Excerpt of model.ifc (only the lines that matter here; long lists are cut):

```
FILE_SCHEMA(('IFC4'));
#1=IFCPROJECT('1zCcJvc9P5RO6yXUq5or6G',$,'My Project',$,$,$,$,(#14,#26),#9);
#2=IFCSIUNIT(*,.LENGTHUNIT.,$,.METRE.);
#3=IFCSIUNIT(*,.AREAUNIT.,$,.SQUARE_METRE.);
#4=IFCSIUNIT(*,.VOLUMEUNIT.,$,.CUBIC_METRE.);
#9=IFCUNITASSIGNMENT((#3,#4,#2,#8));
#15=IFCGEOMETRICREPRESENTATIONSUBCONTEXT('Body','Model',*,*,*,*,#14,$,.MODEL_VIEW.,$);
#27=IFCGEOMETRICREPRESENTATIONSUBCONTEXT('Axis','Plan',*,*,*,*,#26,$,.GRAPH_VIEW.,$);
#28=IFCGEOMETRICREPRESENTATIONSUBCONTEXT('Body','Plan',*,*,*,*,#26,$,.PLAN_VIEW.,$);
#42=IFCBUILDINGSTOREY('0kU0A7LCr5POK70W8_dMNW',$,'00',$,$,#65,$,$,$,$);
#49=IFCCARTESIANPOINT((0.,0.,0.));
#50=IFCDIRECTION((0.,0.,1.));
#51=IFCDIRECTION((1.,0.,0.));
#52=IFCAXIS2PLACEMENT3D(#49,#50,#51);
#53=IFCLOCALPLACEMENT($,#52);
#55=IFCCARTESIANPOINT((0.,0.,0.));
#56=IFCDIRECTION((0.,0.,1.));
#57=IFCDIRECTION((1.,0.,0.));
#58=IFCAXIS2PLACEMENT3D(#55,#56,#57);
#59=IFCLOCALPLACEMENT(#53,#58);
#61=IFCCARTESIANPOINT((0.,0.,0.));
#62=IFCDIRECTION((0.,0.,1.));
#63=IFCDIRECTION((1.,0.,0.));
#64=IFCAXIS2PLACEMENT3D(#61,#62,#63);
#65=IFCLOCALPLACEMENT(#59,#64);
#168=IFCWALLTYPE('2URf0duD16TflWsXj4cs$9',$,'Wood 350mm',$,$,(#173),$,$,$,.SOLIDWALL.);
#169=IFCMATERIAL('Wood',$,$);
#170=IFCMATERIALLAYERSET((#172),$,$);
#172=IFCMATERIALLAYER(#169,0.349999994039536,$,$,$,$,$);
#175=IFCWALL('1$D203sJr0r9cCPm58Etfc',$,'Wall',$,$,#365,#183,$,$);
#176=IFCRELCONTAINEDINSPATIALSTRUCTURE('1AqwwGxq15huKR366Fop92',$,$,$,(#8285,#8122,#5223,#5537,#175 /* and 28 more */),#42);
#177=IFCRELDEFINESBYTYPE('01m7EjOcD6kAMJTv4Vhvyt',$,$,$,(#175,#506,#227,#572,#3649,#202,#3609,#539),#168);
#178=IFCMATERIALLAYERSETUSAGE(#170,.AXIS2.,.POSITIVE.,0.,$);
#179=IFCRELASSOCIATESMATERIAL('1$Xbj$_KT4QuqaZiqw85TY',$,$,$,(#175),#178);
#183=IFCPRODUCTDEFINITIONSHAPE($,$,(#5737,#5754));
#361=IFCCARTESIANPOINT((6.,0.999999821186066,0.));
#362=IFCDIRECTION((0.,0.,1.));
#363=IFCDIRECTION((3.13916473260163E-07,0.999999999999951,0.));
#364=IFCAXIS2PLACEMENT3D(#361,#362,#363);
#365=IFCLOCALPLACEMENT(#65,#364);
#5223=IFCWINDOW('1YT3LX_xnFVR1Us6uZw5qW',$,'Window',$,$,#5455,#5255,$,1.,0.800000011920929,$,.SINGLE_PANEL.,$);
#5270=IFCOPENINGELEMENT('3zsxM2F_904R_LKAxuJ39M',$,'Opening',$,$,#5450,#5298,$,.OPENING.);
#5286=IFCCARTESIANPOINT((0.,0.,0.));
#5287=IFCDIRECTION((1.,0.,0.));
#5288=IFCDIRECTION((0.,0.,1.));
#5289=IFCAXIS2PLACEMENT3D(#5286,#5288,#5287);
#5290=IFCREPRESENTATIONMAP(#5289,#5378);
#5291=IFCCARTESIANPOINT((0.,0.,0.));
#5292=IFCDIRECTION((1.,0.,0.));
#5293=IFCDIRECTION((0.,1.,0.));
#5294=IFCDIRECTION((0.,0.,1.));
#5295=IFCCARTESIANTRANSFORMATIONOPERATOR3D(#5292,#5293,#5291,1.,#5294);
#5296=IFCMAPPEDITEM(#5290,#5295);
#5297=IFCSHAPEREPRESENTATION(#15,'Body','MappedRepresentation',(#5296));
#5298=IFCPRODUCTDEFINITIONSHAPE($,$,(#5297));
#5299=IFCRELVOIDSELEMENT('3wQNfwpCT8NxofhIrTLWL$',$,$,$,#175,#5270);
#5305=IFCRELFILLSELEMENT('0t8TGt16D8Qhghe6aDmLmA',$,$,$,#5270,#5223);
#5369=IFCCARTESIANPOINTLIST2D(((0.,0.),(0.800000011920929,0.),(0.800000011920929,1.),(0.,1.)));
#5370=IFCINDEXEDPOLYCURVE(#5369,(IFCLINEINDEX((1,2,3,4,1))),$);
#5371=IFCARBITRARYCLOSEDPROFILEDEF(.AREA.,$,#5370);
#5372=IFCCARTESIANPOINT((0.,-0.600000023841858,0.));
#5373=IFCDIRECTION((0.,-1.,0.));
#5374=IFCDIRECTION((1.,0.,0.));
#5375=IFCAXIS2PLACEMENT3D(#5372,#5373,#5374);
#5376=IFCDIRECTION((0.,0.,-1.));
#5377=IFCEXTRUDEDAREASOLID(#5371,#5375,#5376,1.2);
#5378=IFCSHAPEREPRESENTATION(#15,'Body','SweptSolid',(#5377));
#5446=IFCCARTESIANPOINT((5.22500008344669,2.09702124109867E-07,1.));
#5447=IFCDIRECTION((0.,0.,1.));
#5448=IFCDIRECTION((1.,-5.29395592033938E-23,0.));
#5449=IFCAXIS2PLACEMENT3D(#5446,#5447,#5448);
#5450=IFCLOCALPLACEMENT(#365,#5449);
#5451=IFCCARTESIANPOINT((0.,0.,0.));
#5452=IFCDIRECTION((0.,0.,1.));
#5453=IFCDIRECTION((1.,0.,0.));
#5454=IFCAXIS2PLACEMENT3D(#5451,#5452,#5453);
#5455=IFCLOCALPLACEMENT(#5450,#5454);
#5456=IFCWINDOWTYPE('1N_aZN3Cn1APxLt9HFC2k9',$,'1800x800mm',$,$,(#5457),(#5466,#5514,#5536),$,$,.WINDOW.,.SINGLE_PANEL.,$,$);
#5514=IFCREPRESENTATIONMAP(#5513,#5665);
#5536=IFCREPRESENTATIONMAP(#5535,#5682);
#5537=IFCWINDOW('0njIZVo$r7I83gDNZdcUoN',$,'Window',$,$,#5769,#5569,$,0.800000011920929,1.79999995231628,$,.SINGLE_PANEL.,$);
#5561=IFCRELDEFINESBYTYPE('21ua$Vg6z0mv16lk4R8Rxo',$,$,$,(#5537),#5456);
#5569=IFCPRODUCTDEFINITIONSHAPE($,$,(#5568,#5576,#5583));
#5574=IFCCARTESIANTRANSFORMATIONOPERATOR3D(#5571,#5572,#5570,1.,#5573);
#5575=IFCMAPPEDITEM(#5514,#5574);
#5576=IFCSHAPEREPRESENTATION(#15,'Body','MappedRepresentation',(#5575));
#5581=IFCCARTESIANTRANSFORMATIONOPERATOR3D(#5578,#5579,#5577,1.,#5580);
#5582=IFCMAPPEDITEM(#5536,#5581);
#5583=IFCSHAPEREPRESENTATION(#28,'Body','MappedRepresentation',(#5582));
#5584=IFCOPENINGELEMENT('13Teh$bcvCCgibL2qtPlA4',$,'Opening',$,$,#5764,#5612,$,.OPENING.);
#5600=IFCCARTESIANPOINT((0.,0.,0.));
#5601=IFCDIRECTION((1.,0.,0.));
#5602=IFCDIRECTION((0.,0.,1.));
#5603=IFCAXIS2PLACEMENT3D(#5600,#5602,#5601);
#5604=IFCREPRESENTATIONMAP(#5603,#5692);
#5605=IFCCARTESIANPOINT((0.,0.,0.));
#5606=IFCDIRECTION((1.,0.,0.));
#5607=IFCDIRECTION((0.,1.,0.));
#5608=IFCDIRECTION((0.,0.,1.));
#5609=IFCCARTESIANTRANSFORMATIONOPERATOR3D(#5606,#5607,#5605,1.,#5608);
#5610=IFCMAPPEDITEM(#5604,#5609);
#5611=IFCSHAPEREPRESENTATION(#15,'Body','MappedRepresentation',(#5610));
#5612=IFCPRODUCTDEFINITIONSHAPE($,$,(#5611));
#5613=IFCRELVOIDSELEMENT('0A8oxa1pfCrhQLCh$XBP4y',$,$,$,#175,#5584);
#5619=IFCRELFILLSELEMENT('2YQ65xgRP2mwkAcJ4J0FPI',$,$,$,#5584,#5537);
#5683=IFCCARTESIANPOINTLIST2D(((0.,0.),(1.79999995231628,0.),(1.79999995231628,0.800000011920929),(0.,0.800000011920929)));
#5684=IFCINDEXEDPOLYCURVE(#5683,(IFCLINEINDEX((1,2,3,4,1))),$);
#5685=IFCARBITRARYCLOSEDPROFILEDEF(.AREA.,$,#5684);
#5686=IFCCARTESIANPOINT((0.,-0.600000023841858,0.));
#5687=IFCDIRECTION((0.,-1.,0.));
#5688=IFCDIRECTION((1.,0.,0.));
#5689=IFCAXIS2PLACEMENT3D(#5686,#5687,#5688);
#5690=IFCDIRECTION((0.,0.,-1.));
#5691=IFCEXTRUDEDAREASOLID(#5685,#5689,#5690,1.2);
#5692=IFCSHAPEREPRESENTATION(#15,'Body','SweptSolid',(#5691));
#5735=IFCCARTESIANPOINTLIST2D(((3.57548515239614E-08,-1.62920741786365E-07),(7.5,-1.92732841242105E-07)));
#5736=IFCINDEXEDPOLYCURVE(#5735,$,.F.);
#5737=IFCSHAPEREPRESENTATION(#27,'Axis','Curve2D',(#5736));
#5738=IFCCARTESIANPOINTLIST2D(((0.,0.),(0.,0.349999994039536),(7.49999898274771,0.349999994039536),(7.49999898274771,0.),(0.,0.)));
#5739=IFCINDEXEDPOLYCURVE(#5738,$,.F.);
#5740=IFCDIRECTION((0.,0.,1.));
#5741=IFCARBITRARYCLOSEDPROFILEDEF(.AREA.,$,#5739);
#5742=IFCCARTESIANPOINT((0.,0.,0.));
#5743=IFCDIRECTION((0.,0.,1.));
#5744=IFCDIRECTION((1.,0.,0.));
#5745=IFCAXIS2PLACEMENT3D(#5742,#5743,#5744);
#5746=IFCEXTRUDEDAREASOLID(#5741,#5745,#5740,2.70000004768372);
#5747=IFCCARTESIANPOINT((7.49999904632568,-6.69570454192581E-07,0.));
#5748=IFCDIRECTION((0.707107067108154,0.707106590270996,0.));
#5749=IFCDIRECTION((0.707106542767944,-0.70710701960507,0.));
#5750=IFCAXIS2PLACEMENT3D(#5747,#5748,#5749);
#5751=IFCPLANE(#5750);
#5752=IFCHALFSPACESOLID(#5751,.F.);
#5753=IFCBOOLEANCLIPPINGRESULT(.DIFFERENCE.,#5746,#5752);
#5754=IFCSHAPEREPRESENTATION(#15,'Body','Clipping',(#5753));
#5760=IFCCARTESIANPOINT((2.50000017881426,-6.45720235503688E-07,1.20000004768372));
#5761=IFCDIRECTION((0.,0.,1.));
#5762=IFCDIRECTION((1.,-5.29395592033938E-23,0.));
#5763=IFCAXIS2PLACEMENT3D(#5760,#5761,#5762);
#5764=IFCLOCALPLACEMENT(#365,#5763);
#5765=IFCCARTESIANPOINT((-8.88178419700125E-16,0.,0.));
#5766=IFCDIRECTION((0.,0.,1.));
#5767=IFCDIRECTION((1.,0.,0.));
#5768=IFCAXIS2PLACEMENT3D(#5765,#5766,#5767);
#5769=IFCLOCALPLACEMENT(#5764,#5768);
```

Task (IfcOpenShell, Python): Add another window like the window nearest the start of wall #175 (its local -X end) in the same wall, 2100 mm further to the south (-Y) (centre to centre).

```python
import ifcopenshell
import ifcopenshell.api.feature
import ifcopenshell.api.geometry
import ifcopenshell.api.root
import ifcopenshell.geom
import ifcopenshell.util.element
import ifcopenshell.util.placement
import ifcopenshell.util.shape

model = ifcopenshell.open("model.ifc")
settings = ifcopenshell.geom.settings()


def volume(element):
    """Net volume in cubic metres, openings subtracted."""
    shape = ifcopenshell.geom.create_shape(settings, element)
    return ifcopenshell.util.shape.get_volume(shape.geometry)


window = model.by_guid("0njIZVo$r7I83gDNZdcUoN")
opening = window.FillsVoids[0].RelatingOpeningElement
wall = opening.VoidsElements[0].RelatingBuildingElement
before = volume(wall)
shift = ifcopenshell.util.placement.get_local_placement(wall.ObjectPlacement)[:3, 0] * -2.1

# copy_class copies the void relationship, type, container and properties, but no geometry.
new_opening = ifcopenshell.api.root.copy_class(model, product=opening)
new_opening.Representation = ifcopenshell.util.element.copy_deep(
    model, opening.Representation, exclude=["IfcGeometricRepresentationContext", "IfcRepresentationMap"]
)
new_window = ifcopenshell.api.root.copy_class(model, product=window)
new_window.Representation = ifcopenshell.util.element.copy_deep(
    model, window.Representation, exclude=["IfcGeometricRepresentationContext", "IfcRepresentationMap"]
)
ifcopenshell.api.feature.add_filling(model, opening=new_opening, element=new_window)

for old, new in ((opening, new_opening), (window, new_window)):
    matrix = ifcopenshell.util.placement.get_local_placement(old.ObjectPlacement)
    matrix[:3, 3] += shift
    ifcopenshell.api.geometry.edit_object_placement(model, product=new, matrix=matrix, is_si=False)

after = volume(wall)

print(f"wall volume {before:.3f} -> {after:.3f} m3")

model.write("model_rev.ifc")
```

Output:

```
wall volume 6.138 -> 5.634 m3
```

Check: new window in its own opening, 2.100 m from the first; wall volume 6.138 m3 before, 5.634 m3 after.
